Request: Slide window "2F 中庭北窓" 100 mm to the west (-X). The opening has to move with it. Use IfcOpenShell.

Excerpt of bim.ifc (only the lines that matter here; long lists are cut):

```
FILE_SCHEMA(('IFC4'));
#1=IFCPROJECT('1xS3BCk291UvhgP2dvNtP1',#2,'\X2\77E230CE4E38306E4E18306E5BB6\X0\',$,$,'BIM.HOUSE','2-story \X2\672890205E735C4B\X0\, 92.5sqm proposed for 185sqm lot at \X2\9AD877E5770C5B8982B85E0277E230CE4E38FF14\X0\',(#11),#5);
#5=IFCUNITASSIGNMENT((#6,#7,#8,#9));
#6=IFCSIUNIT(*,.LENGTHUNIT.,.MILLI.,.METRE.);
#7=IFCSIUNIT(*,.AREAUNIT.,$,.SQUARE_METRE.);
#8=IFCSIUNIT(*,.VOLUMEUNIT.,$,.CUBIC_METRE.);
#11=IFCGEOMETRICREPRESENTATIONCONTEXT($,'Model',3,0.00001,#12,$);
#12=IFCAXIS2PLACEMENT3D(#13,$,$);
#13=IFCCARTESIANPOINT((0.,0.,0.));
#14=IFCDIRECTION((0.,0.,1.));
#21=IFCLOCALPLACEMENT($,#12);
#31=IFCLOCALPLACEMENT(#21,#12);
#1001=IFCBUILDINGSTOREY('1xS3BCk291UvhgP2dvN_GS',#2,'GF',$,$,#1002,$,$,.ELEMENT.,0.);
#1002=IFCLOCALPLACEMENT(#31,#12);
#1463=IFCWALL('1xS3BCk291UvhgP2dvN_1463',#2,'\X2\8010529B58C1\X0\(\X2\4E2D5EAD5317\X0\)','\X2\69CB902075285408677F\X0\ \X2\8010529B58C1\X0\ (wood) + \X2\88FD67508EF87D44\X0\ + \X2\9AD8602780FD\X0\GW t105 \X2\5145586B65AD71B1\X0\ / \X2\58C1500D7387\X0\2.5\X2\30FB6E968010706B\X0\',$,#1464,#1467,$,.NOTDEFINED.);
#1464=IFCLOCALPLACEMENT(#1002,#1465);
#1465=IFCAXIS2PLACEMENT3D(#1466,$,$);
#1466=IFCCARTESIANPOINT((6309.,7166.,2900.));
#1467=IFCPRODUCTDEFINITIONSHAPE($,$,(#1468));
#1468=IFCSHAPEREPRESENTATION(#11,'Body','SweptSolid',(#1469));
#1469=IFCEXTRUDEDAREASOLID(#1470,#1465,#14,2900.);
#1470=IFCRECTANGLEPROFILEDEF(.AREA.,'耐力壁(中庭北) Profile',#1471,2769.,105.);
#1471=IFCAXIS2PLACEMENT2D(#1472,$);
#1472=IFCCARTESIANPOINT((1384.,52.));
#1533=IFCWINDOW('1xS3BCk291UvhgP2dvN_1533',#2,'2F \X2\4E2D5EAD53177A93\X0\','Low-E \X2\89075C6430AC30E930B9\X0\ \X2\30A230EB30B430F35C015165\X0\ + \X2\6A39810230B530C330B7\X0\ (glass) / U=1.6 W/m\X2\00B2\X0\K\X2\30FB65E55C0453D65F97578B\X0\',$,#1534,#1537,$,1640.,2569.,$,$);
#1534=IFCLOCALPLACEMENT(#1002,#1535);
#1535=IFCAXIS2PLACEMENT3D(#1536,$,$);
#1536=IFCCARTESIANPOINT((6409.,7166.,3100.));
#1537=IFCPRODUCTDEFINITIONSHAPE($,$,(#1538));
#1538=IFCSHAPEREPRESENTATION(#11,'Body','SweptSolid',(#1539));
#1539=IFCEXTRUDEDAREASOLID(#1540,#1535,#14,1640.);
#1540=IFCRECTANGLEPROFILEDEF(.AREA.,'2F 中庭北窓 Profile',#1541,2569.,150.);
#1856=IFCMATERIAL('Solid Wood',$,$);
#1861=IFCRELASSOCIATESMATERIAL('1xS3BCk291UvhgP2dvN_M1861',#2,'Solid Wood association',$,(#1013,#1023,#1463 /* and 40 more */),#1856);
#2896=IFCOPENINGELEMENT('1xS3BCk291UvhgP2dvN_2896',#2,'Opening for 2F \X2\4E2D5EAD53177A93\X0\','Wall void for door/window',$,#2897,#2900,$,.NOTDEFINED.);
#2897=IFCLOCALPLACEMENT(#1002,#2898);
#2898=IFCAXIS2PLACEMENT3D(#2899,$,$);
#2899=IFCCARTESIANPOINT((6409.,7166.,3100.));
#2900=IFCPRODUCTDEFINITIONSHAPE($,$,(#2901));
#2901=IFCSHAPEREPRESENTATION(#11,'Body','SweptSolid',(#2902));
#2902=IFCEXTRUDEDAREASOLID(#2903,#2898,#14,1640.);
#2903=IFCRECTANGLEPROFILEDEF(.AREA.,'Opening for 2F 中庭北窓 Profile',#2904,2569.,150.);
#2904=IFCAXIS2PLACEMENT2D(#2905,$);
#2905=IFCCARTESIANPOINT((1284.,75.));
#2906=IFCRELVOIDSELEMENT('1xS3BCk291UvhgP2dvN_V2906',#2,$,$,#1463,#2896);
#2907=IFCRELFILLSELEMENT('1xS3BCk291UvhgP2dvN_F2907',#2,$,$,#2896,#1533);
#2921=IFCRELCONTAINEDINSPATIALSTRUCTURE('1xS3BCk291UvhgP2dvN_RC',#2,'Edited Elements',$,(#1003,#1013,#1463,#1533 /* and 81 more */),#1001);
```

```python
import ifcopenshell
import ifcopenshell.api.geometry
import ifcopenshell.util.placement
import ifcopenshell.util.unit

model = ifcopenshell.open("bim.ifc")
unit_scale = ifcopenshell.util.unit.calculate_unit_scale(model)

window = model.by_guid("1xS3BCk291UvhgP2dvN_1533")
opening = window.FillsVoids[0].RelatingOpeningElement
wall = opening.VoidsElements[0].RelatingBuildingElement

wall_matrix = ifcopenshell.util.placement.get_local_placement(wall.ObjectPlacement)
shift = wall_matrix[:3, 0] * -0.1 / unit_scale
before = ifcopenshell.util.placement.get_local_placement(window.ObjectPlacement)[:3, 3].copy()

# The window is not placed relative to its opening, so move both.
for product in (opening, window):
    matrix = ifcopenshell.util.placement.get_local_placement(product.ObjectPlacement)
    matrix[:3, 3] += shift
    ifcopenshell.api.geometry.edit_object_placement(model, product=product, matrix=matrix, is_si=False)

after = ifcopenshell.util.placement.get_local_placement(window.ObjectPlacement)[:3, 3]
print("window moved by", (after - before).round(3) + 0.0)

model.write("bim_v2.ifc")
```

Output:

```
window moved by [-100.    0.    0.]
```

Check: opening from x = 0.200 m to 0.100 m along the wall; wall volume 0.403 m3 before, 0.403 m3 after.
